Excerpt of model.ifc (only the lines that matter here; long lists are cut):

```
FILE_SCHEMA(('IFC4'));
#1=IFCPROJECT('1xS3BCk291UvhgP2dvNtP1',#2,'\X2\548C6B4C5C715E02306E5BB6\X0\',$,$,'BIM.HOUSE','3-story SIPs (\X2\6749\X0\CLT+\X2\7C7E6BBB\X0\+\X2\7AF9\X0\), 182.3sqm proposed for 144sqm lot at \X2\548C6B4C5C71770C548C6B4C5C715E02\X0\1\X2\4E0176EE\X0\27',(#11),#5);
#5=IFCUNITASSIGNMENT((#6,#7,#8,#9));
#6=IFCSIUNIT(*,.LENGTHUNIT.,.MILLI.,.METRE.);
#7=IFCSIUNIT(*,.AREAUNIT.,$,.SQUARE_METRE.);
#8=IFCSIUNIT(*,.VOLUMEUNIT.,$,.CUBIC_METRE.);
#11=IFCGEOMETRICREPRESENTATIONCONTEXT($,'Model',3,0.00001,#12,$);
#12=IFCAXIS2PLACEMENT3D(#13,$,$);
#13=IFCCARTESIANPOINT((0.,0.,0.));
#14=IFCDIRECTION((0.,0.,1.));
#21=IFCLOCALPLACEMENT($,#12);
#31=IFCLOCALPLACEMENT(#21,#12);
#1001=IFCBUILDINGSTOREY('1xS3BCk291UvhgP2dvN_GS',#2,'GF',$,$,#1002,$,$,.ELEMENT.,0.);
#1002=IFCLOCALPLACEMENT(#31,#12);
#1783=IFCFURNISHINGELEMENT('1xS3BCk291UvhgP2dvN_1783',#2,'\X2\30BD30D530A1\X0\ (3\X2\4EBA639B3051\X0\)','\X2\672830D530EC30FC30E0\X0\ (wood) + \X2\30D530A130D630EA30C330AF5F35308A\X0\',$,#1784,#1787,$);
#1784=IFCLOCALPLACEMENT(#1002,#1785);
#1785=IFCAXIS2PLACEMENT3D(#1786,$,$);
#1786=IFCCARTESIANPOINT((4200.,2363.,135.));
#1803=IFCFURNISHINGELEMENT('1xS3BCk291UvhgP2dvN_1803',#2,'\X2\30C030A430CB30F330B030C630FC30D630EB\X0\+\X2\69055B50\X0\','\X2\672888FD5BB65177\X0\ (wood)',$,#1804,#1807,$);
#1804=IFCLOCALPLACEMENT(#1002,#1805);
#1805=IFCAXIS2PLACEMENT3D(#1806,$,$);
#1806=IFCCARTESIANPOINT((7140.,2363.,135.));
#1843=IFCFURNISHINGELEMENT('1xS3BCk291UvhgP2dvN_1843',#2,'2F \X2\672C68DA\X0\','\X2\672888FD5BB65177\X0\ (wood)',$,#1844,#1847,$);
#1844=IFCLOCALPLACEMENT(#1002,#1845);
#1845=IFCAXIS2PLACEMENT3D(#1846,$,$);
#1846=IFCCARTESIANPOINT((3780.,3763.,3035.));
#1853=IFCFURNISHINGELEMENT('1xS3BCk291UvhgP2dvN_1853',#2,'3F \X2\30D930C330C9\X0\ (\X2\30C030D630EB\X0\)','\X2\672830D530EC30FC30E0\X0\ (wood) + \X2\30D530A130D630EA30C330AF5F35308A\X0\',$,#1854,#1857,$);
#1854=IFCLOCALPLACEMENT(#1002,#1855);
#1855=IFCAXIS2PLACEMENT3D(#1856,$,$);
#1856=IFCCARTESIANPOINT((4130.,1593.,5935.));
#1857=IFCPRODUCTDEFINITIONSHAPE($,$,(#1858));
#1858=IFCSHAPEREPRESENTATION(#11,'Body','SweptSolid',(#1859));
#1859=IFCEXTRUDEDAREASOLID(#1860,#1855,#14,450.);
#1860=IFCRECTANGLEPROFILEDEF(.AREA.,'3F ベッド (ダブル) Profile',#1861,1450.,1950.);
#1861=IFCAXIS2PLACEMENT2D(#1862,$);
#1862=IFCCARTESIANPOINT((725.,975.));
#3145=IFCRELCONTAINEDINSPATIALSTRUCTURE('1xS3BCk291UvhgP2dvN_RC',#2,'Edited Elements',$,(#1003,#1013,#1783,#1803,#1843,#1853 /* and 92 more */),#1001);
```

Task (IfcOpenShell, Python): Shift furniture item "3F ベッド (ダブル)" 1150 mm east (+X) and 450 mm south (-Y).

```python
import ifcopenshell
import ifcopenshell.api.geometry
import ifcopenshell.util.placement
import ifcopenshell.util.unit

model = ifcopenshell.open("model.ifc")
unit_scale = ifcopenshell.util.unit.calculate_unit_scale(model)

item = model.by_id(1853)
matrix = ifcopenshell.util.placement.get_local_placement(item.ObjectPlacement)
matrix[0, 3] += 1.15 / unit_scale
matrix[1, 3] -= 0.45 / unit_scale
ifcopenshell.api.geometry.edit_object_placement(model, product=item, matrix=matrix, is_si=False)

print(ifcopenshell.util.placement.get_local_placement(item.ObjectPlacement).round(3) + 0.0)

model.write("model-out.ifc")
```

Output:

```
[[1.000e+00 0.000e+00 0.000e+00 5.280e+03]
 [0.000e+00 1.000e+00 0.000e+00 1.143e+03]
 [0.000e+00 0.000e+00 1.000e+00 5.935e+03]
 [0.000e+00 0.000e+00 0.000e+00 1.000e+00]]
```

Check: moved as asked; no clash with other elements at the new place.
